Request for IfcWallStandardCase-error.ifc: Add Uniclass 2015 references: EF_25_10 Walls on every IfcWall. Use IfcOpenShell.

First a look at what the model holds.

```python
import ifcopenshell

model = ifcopenshell.open("IfcWallStandardCase-error.ifc")
print(model.schema)
print("classifications:", [c.Name for c in model.by_type("IfcClassification")])
for ifc_class in ("IfcDoor", "IfcRoof", "IfcStair", "IfcWall", "IfcWindow"):
    print(ifc_class, len(model.by_type(ifc_class)))
```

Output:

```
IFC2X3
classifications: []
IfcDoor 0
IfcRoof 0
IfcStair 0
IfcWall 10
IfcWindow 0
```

```python
import ifcopenshell
import ifcopenshell.api.classification

model = ifcopenshell.open("IfcWallStandardCase-error.ifc")

# IFC2X3 requires Source and Edition and has no link from the project to the system.
system = model.create_entity("IfcClassification", Source="NBS", Edition="2015", Name="Uniclass 2015")

codes = {
    "IfcWall": ("EF_25_10", "Walls"),
}
for ifc_class, (code, name) in codes.items():
    products = model.by_type(ifc_class)
    ifcopenshell.api.classification.add_reference(
        model, products=products, classification=system, identification=code, name=name
    )
    print(code, len(products))

model.write("IfcWallStandardCase-error_v2.ifc")
```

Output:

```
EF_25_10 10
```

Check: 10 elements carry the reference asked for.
